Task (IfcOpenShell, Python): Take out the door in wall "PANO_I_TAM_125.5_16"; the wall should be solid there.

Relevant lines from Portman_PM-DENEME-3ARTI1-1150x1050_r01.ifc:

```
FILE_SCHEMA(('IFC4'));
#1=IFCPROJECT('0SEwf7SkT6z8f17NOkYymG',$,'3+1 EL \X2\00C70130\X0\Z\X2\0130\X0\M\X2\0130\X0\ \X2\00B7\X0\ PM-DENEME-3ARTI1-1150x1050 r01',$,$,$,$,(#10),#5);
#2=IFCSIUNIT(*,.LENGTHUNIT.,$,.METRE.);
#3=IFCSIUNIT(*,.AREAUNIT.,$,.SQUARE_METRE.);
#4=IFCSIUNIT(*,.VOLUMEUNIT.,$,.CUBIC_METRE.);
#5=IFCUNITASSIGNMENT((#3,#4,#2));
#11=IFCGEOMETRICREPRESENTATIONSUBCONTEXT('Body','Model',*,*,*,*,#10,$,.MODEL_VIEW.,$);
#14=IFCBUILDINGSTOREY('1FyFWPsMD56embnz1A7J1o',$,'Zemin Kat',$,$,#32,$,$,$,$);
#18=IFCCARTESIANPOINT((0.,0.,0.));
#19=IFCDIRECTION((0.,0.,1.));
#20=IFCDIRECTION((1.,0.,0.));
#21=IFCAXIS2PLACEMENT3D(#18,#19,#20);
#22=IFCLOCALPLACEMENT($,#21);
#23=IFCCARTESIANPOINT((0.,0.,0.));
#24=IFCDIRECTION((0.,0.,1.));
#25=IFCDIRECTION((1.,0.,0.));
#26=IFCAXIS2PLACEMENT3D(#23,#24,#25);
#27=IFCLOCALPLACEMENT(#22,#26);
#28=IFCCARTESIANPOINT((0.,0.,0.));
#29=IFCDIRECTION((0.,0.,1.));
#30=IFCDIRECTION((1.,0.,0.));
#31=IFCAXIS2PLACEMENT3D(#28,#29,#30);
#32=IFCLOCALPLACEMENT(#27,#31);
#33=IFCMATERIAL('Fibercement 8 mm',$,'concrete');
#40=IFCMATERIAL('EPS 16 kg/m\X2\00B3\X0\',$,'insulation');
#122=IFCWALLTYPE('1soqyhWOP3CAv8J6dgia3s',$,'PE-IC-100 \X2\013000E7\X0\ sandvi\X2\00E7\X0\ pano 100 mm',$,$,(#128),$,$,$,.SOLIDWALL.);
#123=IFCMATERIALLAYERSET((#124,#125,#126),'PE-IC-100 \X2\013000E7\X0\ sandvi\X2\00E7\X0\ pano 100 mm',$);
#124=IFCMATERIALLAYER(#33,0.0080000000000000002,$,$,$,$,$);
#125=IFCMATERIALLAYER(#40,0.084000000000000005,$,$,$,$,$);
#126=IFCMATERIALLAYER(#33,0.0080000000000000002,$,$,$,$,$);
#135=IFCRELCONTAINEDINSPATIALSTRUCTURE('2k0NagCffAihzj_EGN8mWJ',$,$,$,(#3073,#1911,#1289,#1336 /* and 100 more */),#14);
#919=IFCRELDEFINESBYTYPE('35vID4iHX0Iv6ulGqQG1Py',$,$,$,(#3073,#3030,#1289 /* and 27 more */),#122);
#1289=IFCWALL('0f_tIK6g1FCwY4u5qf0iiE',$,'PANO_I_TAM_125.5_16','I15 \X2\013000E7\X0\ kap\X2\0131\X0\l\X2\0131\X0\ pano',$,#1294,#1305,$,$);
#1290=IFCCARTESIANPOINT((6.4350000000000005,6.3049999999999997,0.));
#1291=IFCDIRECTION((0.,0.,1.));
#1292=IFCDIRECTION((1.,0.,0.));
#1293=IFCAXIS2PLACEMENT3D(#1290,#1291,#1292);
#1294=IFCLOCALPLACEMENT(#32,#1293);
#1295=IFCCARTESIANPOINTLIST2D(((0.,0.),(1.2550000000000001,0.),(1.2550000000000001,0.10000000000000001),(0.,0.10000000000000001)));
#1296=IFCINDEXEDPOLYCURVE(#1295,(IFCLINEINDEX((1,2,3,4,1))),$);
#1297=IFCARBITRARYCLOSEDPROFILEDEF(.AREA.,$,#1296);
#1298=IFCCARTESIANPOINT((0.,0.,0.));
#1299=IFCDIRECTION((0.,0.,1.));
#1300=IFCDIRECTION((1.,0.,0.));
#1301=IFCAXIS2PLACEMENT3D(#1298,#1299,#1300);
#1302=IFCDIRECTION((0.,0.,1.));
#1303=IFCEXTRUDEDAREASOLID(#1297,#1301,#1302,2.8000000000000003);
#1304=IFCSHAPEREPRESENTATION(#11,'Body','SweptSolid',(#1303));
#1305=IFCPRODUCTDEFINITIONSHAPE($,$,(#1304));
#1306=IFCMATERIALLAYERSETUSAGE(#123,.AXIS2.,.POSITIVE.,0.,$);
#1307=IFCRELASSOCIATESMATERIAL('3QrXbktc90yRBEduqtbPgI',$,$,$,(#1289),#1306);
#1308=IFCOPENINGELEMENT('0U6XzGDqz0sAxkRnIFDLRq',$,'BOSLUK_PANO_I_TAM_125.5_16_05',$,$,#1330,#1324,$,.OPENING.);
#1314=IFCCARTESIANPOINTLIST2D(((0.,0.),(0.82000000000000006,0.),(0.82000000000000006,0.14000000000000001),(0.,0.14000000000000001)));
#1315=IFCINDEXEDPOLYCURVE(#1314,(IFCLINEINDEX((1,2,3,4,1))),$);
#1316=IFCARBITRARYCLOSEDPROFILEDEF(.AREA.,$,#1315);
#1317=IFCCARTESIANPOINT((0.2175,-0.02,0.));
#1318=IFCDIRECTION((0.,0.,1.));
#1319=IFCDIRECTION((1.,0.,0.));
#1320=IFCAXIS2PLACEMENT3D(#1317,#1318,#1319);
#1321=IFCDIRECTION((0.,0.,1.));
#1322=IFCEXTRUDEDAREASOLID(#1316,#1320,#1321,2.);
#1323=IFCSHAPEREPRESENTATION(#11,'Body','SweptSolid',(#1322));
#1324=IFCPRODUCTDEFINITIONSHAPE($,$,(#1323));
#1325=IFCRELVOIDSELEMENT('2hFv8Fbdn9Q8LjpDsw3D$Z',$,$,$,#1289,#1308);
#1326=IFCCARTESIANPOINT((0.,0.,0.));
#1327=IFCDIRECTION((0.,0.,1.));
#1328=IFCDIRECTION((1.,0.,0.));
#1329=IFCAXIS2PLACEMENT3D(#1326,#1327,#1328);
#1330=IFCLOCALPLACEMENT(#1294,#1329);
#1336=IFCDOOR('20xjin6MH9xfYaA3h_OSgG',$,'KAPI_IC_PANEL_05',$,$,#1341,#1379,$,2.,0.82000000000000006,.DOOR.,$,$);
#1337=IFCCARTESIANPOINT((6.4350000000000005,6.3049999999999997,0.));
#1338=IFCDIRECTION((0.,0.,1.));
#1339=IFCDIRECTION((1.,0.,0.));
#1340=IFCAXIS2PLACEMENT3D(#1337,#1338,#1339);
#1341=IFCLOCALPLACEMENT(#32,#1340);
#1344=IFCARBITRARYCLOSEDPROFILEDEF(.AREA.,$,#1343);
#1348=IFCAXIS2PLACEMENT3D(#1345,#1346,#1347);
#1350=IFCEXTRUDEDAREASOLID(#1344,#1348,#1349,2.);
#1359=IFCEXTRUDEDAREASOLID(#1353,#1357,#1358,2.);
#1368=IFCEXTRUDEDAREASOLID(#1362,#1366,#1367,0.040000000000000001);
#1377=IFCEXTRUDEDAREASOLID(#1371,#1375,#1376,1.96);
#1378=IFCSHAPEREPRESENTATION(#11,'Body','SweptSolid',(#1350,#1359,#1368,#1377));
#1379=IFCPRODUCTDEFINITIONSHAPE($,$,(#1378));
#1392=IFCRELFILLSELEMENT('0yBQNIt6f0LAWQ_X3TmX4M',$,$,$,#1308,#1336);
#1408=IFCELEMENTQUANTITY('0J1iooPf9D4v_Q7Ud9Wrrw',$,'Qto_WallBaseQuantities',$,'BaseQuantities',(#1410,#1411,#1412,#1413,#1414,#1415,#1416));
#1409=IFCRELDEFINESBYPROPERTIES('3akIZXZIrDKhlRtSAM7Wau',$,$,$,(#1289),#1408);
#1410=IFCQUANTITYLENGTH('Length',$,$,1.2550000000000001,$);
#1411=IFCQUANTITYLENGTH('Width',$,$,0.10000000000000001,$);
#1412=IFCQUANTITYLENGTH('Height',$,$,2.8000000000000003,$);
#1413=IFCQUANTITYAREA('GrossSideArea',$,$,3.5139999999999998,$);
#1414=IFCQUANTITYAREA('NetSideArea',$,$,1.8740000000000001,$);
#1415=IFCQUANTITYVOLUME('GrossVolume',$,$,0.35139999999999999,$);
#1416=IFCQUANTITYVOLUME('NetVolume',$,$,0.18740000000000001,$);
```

```python
import ifcopenshell
import ifcopenshell.api.feature
import ifcopenshell.api.pset
import ifcopenshell.api.root
import ifcopenshell.geom
import ifcopenshell.util.element
import ifcopenshell.util.shape
import ifcopenshell.util.unit

model = ifcopenshell.open("Portman_PM-DENEME-3ARTI1-1150x1050_r01.ifc")
area_scale = ifcopenshell.util.unit.calculate_unit_scale(model, "AREAUNIT")
volume_scale = ifcopenshell.util.unit.calculate_unit_scale(model, "VOLUMEUNIT")
settings = ifcopenshell.geom.settings()


def volume(element):
    """Net volume in cubic metres, openings subtracted."""
    shape = ifcopenshell.geom.create_shape(settings, element)
    return ifcopenshell.util.shape.get_volume(shape.geometry)


door = model.by_guid("20xjin6MH9xfYaA3h_OSgG")
opening = door.FillsVoids[0].RelatingOpeningElement
wall = opening.VoidsElements[0].RelatingBuildingElement
before = volume(wall)

ifcopenshell.api.root.remove_product(model, product=door)
ifcopenshell.api.feature.remove_feature(model, feature=opening)

after = volume(wall)
thickness = 0.1  # wall thickness in metres

# Update the wall's stored quantities.
qto = model.by_id(ifcopenshell.util.element.get_pset(wall, "Qto_WallBaseQuantities", should_inherit=False)["id"])
ifcopenshell.api.pset.edit_qto(model, qto=qto, properties={
    "NetSideArea": after / thickness / area_scale,
    "NetVolume": after / volume_scale,
})

print(f"wall volume {before:.3f} -> {after:.3f} m3")

model.write("Portman_PM-DENEME-3ARTI1-1150x1050_r01_v2.ifc")
```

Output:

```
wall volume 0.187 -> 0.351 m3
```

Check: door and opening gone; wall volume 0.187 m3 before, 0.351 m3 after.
